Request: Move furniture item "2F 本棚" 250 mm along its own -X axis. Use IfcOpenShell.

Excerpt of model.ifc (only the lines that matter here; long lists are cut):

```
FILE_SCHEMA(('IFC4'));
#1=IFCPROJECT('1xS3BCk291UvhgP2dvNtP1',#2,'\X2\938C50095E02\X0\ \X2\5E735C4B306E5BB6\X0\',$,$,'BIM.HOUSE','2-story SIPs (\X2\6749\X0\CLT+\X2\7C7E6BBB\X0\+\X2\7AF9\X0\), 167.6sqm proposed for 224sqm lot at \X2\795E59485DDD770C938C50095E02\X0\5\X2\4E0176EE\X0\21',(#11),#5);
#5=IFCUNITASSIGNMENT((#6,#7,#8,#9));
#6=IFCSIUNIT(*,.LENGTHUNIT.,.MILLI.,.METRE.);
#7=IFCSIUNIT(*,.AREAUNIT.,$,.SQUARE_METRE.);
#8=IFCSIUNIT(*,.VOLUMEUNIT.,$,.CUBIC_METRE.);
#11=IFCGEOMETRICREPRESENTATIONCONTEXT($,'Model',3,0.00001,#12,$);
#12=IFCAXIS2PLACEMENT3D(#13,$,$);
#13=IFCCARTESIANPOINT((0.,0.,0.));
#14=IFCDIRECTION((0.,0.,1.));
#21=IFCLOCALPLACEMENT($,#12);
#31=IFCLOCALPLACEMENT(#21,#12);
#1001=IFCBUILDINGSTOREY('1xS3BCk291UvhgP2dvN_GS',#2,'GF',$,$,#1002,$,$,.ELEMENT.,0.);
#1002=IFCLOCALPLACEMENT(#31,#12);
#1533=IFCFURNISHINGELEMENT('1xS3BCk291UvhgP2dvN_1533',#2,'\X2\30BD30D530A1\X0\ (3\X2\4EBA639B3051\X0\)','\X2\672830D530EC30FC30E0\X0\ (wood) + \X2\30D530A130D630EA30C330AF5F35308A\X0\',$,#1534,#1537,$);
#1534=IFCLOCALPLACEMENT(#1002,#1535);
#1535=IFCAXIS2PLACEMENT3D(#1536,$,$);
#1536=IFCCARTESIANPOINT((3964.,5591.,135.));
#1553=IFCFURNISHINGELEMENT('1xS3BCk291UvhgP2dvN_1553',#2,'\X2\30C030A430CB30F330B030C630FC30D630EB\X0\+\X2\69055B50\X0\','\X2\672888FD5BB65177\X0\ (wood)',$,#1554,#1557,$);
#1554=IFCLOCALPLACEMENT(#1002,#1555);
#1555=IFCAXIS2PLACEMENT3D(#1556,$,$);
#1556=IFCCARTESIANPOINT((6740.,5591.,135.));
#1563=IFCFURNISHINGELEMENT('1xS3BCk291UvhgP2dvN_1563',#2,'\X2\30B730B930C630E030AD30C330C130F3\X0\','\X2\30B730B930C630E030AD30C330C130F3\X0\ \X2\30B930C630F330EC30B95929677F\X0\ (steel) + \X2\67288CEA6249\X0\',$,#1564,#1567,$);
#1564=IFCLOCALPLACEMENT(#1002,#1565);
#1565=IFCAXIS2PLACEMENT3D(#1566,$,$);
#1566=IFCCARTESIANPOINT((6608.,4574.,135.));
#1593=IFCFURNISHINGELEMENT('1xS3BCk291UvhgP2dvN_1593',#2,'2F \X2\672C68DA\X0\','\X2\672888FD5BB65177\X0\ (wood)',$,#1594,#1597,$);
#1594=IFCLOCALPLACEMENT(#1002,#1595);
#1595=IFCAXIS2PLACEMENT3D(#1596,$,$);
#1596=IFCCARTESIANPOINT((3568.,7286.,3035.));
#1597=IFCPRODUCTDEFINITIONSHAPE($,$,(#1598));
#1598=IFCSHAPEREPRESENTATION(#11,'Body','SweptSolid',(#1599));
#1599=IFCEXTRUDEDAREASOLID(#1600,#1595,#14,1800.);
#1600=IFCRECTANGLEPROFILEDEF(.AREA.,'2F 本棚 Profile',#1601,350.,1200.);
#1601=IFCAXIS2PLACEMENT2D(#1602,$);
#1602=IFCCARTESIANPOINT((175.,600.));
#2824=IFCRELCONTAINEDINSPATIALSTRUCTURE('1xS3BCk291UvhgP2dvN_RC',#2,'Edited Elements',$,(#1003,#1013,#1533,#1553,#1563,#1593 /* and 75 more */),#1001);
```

```python
import ifcopenshell
import ifcopenshell.api.geometry
import ifcopenshell.util.placement
import ifcopenshell.util.unit

model = ifcopenshell.open("model.ifc")
unit_scale = ifcopenshell.util.unit.calculate_unit_scale(model)

item = model.by_id(1593)
matrix = ifcopenshell.util.placement.get_local_placement(item.ObjectPlacement)
matrix[:3, 3] -= matrix[:3, 0] * 0.25 / unit_scale
ifcopenshell.api.geometry.edit_object_placement(model, product=item, matrix=matrix, is_si=False)

print(ifcopenshell.util.placement.get_local_placement(item.ObjectPlacement).round(3) + 0.0)

model.write("model_v2.ifc")
```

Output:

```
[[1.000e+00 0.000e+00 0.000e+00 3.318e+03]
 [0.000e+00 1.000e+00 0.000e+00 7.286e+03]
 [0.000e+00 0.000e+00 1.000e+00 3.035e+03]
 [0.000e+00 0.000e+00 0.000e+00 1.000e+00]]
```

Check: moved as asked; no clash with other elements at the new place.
